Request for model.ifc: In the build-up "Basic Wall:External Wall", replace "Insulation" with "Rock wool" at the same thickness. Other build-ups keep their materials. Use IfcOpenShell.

First a look at what the model holds.

```python
import ifcopenshell
import ifcopenshell.util.element

model = ifcopenshell.open("model.ifc")
print(model.schema)
for layer_set in model.by_type("IfcMaterialLayerSet"):
    if layer_set.LayerSetName == "Basic Wall:External Wall":
        for layer in layer_set.MaterialLayers:
            print(layer.id(), layer.Material and layer.Material.Name, layer.LayerThickness, sep=" | ")
        print(len(ifcopenshell.util.element.get_elements_by_material(model, layer_set)), "elements and types use it")
print(sorted(m.Name for m in model.by_type("IfcMaterial") if m.Name)[:60])
```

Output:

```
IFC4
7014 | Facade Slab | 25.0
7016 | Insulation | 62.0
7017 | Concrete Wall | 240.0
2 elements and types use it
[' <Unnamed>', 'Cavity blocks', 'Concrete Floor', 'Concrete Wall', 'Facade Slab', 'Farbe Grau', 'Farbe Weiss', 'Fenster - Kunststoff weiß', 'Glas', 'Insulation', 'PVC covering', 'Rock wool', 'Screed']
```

```python
import ifcopenshell
import ifcopenshell.api.material

model = ifcopenshell.open("model.ifc")

layer_set = next(s for s in model.by_type("IfcMaterialLayerSet") if s.LayerSetName == "Basic Wall:External Wall")
layer = next(l for l in layer_set.MaterialLayers if l.Material and l.Material.Name == "Insulation")
material = next(m for m in model.by_type("IfcMaterial") if m.Name == "Rock wool")

# Point this one layer at the other material; renaming the old one would change it everywhere.
ifcopenshell.api.material.edit_layer(model, layer=layer, attributes={}, material=material)

print([l.Material.Name if l.Material else None for l in layer_set.MaterialLayers])

model.write("model_edited.ifc")
```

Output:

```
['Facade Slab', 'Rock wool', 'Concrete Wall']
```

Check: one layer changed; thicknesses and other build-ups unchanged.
